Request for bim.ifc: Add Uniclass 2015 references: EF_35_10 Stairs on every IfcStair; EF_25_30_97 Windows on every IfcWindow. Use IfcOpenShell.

First a look at what the model holds.

```python
import ifcopenshell

model = ifcopenshell.open("bim.ifc")
print(model.schema)
print("classifications:", [c.Name for c in model.by_type("IfcClassification")])
for ifc_class in ("IfcDoor", "IfcRoof", "IfcStair", "IfcWall", "IfcWindow"):
    print(ifc_class, len(model.by_type(ifc_class)))
```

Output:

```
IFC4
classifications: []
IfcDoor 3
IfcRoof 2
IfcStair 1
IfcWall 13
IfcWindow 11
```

```python
import ifcopenshell
import ifcopenshell.api.classification

model = ifcopenshell.open("bim.ifc")

system = ifcopenshell.api.classification.add_classification(model, classification="Uniclass 2015")

codes = {
    "IfcStair": ("EF_35_10", "Stairs"),
    "IfcWindow": ("EF_25_30_97", "Windows"),
}
for ifc_class, (code, name) in codes.items():
    products = model.by_type(ifc_class)
    ifcopenshell.api.classification.add_reference(
        model, products=products, classification=system, identification=code, name=name
    )
    print(code, len(products))

model.write("bim_v2.ifc")
```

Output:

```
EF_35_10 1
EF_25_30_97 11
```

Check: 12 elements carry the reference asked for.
